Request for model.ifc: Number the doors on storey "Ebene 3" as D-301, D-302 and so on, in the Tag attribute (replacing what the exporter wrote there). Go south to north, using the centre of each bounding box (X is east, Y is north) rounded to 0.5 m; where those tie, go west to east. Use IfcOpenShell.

First a look at what the model holds.

```python
import ifcopenshell
import ifcopenshell.util.element
import ifcopenshell.util.placement

model = ifcopenshell.open("model.ifc")
print(model.schema)
storey = next(s for s in model.by_type("IfcBuildingStorey") if s.Name == "Ebene 3")
doors = [e for e in ifcopenshell.util.element.get_decomposition(storey) if e.is_a("IfcDoor")]
for e in sorted(doors, key=lambda e: e.id()):
    origin = ifcopenshell.util.placement.get_local_placement(e.ObjectPlacement)[:3, 3]
    print(e.id(), e.Tag, e.Name, origin.round(2) + 0.0, sep=" | ")
```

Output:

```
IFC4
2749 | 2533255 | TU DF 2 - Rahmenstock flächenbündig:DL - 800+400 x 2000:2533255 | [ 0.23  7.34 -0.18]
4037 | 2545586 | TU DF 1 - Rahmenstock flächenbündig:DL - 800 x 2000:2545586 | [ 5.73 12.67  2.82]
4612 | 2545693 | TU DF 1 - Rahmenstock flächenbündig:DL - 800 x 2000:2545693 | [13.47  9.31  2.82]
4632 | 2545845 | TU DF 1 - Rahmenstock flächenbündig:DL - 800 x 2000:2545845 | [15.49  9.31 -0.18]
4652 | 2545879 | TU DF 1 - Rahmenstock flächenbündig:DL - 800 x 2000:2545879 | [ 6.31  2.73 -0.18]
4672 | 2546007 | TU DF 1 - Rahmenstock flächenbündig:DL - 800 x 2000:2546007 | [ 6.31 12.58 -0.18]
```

```python
import ifcopenshell
import ifcopenshell.geom
import ifcopenshell.util.element
import ifcopenshell.util.shape

model = ifcopenshell.open("model.ifc")
settings = ifcopenshell.geom.settings()
settings.set("use-world-coords", True)


def centre(element):
    shape = ifcopenshell.geom.create_shape(settings, element)
    return ifcopenshell.util.shape.get_bbox_centroid(shape.geometry)


storey = next(s for s in model.by_type("IfcBuildingStorey") if s.Name == "Ebene 3")
doors = [e for e in ifcopenshell.util.element.get_decomposition(storey) if e.is_a("IfcDoor")]

# Insertion points can sit at a corner or the storey origin, so sort by the geometry (in metres).
centres = {e: centre(e) for e in doors}
doors.sort(key=lambda e: (round(centres[e][1] / 0.5), centres[e][0]))

for i, e in enumerate(doors, start=1):
    number = f"D-3{i:02d}"
    e.Tag = number
    print(e.id(), number)

model.write("model_edited.ifc")
```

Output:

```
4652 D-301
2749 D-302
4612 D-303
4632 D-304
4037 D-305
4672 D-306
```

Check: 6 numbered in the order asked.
